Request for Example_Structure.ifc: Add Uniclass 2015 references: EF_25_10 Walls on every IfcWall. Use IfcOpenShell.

First a look at what the model holds.

```python
import ifcopenshell

model = ifcopenshell.open("Example_Structure.ifc")
print(model.schema)
print("classifications:", [c.Name for c in model.by_type("IfcClassification")])
for ifc_class in ("IfcDoor", "IfcRoof", "IfcStair", "IfcWall", "IfcWindow"):
    print(ifc_class, len(model.by_type(ifc_class)))
```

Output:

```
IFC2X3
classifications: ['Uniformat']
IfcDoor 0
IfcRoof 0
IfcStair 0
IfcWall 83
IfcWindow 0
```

```python
import ifcopenshell
import ifcopenshell.api.classification

model = ifcopenshell.open("Example_Structure.ifc")

# IFC2X3 requires Source and Edition and has no link from the project to the system.
system = model.create_entity("IfcClassification", Source="NBS", Edition="2015", Name="Uniclass 2015")

codes = {
    "IfcWall": ("EF_25_10", "Walls"),
}
for ifc_class, (code, name) in codes.items():
    products = model.by_type(ifc_class)
    ifcopenshell.api.classification.add_reference(
        model, products=products, classification=system, identification=code, name=name
    )
    print(code, len(products))

model.write("Example_Structure-out.ifc")
```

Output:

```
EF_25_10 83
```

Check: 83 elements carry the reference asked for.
